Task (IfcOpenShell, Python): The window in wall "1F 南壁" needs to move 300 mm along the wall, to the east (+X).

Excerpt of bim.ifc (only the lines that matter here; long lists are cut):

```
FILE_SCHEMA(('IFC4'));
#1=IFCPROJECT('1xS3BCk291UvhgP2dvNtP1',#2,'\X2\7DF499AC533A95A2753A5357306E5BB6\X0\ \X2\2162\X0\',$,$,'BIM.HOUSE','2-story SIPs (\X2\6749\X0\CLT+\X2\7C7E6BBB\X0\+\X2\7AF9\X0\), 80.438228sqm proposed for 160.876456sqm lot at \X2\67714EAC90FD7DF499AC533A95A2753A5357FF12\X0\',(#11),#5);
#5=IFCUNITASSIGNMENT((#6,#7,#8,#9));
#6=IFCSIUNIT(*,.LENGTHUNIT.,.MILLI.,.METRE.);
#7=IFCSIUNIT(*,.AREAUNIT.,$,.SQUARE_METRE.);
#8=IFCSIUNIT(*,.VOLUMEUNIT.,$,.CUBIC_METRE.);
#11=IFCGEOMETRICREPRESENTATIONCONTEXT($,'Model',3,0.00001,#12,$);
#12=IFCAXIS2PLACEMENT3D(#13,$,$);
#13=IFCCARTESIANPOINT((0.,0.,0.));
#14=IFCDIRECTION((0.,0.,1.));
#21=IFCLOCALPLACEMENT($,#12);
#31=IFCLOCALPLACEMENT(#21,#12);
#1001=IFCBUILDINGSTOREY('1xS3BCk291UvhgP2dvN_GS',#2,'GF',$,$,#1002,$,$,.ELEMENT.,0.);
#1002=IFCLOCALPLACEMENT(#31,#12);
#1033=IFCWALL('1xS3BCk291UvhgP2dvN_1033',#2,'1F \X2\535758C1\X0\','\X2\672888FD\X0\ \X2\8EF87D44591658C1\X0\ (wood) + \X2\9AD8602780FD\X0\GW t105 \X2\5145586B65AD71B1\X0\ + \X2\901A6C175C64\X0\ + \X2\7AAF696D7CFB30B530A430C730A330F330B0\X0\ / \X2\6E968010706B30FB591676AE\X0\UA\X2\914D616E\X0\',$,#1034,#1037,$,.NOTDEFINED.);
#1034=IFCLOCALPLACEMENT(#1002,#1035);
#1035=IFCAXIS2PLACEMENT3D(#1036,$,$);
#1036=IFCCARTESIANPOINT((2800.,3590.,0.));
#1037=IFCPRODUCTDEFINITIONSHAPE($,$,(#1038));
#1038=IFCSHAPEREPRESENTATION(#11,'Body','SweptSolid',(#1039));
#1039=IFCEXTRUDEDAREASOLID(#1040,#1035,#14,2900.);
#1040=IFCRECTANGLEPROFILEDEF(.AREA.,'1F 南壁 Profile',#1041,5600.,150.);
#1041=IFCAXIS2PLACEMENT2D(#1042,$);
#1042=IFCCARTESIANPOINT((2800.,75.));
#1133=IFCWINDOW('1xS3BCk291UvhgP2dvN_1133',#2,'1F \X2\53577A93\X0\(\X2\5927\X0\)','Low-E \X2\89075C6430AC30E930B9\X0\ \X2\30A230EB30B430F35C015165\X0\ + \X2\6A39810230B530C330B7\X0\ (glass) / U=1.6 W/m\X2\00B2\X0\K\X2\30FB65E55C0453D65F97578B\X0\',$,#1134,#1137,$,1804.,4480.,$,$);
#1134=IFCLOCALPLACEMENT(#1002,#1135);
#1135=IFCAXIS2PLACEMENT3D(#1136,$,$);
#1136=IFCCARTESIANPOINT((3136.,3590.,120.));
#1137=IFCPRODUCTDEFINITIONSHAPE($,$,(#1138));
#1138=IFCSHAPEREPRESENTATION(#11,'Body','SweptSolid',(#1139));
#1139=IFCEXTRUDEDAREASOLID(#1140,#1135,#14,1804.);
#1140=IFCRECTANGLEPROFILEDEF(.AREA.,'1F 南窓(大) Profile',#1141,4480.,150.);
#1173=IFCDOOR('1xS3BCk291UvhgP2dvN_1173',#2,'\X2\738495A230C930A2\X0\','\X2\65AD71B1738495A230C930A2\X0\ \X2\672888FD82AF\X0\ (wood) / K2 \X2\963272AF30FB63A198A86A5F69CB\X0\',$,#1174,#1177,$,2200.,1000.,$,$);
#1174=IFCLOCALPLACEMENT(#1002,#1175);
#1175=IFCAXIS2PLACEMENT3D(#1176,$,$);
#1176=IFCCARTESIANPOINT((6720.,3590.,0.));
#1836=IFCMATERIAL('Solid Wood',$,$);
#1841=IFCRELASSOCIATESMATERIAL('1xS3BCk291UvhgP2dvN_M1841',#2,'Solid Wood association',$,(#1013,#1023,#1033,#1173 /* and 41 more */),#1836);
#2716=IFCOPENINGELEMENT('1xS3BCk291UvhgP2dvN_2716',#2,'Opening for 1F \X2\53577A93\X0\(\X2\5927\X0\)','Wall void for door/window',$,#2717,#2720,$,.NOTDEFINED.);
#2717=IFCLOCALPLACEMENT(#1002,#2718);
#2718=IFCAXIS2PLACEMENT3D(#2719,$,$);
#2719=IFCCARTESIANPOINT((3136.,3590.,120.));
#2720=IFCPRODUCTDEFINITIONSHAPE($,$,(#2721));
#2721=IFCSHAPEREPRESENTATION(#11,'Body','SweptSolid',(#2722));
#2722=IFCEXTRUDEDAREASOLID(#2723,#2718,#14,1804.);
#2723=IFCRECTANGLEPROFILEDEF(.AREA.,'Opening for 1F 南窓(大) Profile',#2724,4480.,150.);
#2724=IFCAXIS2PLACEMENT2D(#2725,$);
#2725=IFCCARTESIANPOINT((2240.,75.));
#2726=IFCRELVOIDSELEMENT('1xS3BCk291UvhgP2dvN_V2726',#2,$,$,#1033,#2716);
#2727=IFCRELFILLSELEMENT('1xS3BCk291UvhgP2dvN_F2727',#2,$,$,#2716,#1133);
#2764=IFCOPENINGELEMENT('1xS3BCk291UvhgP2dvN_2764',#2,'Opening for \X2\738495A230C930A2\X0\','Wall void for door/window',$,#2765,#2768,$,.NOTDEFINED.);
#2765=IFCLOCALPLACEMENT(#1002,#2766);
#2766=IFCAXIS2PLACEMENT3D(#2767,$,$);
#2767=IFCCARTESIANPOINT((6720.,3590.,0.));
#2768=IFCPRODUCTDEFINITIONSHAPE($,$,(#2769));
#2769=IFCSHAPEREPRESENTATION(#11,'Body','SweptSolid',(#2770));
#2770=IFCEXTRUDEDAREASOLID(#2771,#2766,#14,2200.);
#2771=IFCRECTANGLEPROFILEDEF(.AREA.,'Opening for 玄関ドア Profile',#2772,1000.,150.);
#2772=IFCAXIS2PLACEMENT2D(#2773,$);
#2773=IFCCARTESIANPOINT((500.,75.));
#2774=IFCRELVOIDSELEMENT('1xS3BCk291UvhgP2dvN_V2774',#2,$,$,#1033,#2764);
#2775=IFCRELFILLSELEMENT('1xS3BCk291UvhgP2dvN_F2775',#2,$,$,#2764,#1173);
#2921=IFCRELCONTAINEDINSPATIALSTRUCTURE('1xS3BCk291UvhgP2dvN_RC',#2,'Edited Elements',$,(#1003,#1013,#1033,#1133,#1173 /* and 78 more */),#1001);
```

```python
import ifcopenshell
import ifcopenshell.api.geometry
import ifcopenshell.util.placement

model = ifcopenshell.open("bim.ifc")

window = model.by_guid("1xS3BCk291UvhgP2dvN_1133")
opening = window.FillsVoids[0].RelatingOpeningElement
wall = opening.VoidsElements[0].RelatingBuildingElement

wall_matrix = ifcopenshell.util.placement.get_local_placement(wall.ObjectPlacement)
shift = wall_matrix[:3, 0] * 300.0
before = ifcopenshell.util.placement.get_local_placement(window.ObjectPlacement)[:3, 3].copy()

# The window is not placed relative to its opening, so move both.
for product in (opening, window):
    matrix = ifcopenshell.util.placement.get_local_placement(product.ObjectPlacement)
    matrix[:3, 3] += shift
    ifcopenshell.api.geometry.edit_object_placement(model, product=product, matrix=matrix, is_si=False)

after = ifcopenshell.util.placement.get_local_placement(window.ObjectPlacement)[:3, 3]
print("window moved by", (after - before).round(3) + 0.0)

model.write("bim_rev.ifc")
```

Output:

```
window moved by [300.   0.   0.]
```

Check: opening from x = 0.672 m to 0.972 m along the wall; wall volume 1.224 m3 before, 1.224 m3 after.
